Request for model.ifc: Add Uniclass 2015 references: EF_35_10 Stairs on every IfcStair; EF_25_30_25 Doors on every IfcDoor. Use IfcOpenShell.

First a look at what the model holds.

```python
import ifcopenshell

model = ifcopenshell.open("model.ifc")
print(model.schema)
print("classifications:", [c.Name for c in model.by_type("IfcClassification")])
for ifc_class in ("IfcDoor", "IfcRoof", "IfcStair", "IfcWall", "IfcWindow"):
    print(ifc_class, len(model.by_type(ifc_class)))
```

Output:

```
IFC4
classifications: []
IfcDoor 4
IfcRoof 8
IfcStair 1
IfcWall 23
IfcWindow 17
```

```python
import ifcopenshell
import ifcopenshell.api.classification

model = ifcopenshell.open("model.ifc")

system = ifcopenshell.api.classification.add_classification(model, classification="Uniclass 2015")

codes = {
    "IfcStair": ("EF_35_10", "Stairs"),
    "IfcDoor": ("EF_25_30_25", "Doors"),
}
for ifc_class, (code, name) in codes.items():
    products = model.by_type(ifc_class)
    ifcopenshell.api.classification.add_reference(
        model, products=products, classification=system, identification=code, name=name
    )
    print(code, len(products))

model.write("model_updated.ifc")
```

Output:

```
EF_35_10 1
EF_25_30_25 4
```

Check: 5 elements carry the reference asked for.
